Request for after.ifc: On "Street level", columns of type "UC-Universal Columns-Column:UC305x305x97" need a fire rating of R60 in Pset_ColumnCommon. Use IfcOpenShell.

First a look at what the model holds.

```python
import ifcopenshell
import ifcopenshell.util.element

model = ifcopenshell.open("after.ifc")
print(model.schema)
storey = next(s for s in model.by_type("IfcBuildingStorey") if s.Name == "Street level")
columns = [e for e in ifcopenshell.util.element.get_decomposition(storey) if e.is_a("IfcColumn")]
seen = {}
for e in columns:
    element_type = ifcopenshell.util.element.get_type(e)
    key = (element_type.Name if element_type != e and element_type else None, ifcopenshell.util.element.get_pset(e, "Pset_ColumnCommon", "FireRating"))
    seen[key] = seen.get(key, 0) + 1
for (name, value), count in sorted(seen.items(), key=str):
    print(count, "x", name, "|", value)
```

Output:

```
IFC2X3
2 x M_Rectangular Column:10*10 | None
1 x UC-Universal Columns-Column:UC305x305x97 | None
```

```python
import ifcopenshell
import ifcopenshell.api.pset
import ifcopenshell.util.element

model = ifcopenshell.open("after.ifc")

storey = next(s for s in model.by_type("IfcBuildingStorey") if s.Name == "Street level")
columns = [e for e in ifcopenshell.util.element.get_decomposition(storey) if e.is_a("IfcColumn")]

count = 0
for e in columns:
    element_type = ifcopenshell.util.element.get_type(e)
    if element_type in (None, e) or element_type.Name != "UC-Universal Columns-Column:UC305x305x97":
        continue
    # add_pset returns the element's existing set when there is one.
    pset = ifcopenshell.api.pset.add_pset(model, product=e, name="Pset_ColumnCommon")
    ifcopenshell.api.pset.edit_pset(model, pset=pset, properties={"FireRating": "R60"})
    count += 1

print(count, "columns updated")

model.write("after_rev.ifc")
```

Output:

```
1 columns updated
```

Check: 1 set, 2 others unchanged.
